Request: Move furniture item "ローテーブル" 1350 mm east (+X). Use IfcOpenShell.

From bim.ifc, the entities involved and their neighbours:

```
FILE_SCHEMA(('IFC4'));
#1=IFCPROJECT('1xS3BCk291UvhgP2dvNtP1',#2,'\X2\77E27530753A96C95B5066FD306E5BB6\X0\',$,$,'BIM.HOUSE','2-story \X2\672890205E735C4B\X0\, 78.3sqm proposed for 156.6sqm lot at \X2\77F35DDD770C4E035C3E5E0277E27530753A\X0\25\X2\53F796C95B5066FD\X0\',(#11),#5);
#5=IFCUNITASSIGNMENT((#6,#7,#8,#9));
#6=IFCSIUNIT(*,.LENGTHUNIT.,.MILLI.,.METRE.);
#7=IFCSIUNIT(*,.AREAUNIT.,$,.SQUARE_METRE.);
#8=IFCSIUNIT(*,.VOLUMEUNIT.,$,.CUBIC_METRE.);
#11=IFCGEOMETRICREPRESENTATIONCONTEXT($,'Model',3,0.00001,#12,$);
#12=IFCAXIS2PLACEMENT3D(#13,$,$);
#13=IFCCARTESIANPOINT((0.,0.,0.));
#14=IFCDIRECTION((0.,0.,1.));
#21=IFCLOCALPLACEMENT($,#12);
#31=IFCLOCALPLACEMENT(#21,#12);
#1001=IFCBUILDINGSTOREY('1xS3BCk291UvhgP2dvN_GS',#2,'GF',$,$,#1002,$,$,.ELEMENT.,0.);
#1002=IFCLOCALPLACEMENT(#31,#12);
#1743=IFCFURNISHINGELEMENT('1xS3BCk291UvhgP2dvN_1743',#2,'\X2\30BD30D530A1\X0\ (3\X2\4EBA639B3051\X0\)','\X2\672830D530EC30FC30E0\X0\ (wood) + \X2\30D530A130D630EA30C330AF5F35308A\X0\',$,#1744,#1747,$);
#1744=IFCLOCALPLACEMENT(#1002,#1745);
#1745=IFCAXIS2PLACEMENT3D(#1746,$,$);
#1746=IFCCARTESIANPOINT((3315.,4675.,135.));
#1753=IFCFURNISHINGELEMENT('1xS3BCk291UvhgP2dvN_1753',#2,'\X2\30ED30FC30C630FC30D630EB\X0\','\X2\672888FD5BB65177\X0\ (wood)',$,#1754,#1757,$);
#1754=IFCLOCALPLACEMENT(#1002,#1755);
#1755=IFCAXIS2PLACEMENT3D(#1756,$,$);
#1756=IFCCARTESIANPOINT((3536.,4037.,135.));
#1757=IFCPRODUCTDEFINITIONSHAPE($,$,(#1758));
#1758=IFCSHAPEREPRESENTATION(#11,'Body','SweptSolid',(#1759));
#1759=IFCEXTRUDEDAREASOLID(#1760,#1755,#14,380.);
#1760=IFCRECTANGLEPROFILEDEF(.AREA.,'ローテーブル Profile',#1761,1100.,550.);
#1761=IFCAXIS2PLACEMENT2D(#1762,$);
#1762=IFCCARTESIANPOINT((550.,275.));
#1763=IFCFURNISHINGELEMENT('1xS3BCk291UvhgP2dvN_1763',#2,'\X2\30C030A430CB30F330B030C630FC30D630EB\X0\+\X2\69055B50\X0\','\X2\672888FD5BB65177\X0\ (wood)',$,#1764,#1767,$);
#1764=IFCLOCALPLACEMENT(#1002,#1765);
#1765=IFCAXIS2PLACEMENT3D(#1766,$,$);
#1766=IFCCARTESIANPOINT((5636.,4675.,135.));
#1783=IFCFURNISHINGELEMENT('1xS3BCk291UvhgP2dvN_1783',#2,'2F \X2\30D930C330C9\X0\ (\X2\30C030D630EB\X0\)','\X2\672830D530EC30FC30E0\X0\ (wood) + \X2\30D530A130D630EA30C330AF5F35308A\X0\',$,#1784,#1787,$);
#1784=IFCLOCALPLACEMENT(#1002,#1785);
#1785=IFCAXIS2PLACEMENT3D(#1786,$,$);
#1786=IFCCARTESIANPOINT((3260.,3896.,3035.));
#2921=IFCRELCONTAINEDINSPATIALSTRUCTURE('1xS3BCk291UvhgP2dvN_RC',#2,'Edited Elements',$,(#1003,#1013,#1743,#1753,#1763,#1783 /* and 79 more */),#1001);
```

```python
import ifcopenshell
import ifcopenshell.api.geometry
import ifcopenshell.util.placement
import ifcopenshell.util.unit

model = ifcopenshell.open("bim.ifc")
unit_scale = ifcopenshell.util.unit.calculate_unit_scale(model)

item = model.by_guid("1xS3BCk291UvhgP2dvN_1753")
matrix = ifcopenshell.util.placement.get_local_placement(item.ObjectPlacement)
matrix[0, 3] += 1.35 / unit_scale
ifcopenshell.api.geometry.edit_object_placement(model, product=item, matrix=matrix, is_si=False)

print(ifcopenshell.util.placement.get_local_placement(item.ObjectPlacement).round(3) + 0.0)

model.write("bim_updated.ifc")
```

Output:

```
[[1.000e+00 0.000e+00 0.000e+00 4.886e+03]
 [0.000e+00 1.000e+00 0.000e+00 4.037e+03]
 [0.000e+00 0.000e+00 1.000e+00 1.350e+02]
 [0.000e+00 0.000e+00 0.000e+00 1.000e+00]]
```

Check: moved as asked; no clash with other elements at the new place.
